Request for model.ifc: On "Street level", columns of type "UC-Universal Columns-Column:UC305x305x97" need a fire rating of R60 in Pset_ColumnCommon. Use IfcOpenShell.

First a look at what the model holds.

```python
import ifcopenshell
import ifcopenshell.util.element

model = ifcopenshell.open("model.ifc")
print(model.schema)
storey = next(s for s in model.by_type("IfcBuildingStorey") if s.Name == "Street level")
columns = [e for e in ifcopenshell.util.element.get_decomposition(storey) if e.is_a("IfcColumn")]
seen = {}
for e in columns:
    element_type = ifcopenshell.util.element.get_type(e)
    key = (element_type.Name if element_type != e and element_type else None, ifcopenshell.util.element.get_pset(e, "Pset_ColumnCommon", "FireRating"))
    seen[key] = seen.get(key, 0) + 1
for (name, value), count in sorted(seen.items(), key=str):
    print(count, "x", name, "|", value)
```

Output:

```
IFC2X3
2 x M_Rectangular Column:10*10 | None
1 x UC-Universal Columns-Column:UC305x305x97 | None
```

```python
import ifcopenshell
import ifcopenshell.api.pset
import ifcopenshell.util.element

model = ifcopenshell.open("model.ifc")

storey = next(s for s in model.by_type("IfcBuildingStorey") if s.Name == "Street level")
columns = [e for e in ifcopenshell.util.element.get_decomposition(storey) if e.is_a("IfcColumn")]

count = 0
for e in columns:
    element_type = ifcopenshell.util.element.get_type(e)
    if element_type in (None, e) or element_type.Name != "UC-Universal Columns-Column:UC305x305x97":
        continue
    # add_pset returns the element's existing set when there is one.
    pset = ifcopenshell.api.pset.add_pset(model, product=e, name="Pset_ColumnCommon")
    ifcopenshell.api.pset.edit_pset(model, pset=pset, properties={"FireRating": "R60"})
    count += 1

print(count, "columns updated")

model.write("model_edited.ifc")
```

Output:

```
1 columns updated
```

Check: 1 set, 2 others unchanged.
